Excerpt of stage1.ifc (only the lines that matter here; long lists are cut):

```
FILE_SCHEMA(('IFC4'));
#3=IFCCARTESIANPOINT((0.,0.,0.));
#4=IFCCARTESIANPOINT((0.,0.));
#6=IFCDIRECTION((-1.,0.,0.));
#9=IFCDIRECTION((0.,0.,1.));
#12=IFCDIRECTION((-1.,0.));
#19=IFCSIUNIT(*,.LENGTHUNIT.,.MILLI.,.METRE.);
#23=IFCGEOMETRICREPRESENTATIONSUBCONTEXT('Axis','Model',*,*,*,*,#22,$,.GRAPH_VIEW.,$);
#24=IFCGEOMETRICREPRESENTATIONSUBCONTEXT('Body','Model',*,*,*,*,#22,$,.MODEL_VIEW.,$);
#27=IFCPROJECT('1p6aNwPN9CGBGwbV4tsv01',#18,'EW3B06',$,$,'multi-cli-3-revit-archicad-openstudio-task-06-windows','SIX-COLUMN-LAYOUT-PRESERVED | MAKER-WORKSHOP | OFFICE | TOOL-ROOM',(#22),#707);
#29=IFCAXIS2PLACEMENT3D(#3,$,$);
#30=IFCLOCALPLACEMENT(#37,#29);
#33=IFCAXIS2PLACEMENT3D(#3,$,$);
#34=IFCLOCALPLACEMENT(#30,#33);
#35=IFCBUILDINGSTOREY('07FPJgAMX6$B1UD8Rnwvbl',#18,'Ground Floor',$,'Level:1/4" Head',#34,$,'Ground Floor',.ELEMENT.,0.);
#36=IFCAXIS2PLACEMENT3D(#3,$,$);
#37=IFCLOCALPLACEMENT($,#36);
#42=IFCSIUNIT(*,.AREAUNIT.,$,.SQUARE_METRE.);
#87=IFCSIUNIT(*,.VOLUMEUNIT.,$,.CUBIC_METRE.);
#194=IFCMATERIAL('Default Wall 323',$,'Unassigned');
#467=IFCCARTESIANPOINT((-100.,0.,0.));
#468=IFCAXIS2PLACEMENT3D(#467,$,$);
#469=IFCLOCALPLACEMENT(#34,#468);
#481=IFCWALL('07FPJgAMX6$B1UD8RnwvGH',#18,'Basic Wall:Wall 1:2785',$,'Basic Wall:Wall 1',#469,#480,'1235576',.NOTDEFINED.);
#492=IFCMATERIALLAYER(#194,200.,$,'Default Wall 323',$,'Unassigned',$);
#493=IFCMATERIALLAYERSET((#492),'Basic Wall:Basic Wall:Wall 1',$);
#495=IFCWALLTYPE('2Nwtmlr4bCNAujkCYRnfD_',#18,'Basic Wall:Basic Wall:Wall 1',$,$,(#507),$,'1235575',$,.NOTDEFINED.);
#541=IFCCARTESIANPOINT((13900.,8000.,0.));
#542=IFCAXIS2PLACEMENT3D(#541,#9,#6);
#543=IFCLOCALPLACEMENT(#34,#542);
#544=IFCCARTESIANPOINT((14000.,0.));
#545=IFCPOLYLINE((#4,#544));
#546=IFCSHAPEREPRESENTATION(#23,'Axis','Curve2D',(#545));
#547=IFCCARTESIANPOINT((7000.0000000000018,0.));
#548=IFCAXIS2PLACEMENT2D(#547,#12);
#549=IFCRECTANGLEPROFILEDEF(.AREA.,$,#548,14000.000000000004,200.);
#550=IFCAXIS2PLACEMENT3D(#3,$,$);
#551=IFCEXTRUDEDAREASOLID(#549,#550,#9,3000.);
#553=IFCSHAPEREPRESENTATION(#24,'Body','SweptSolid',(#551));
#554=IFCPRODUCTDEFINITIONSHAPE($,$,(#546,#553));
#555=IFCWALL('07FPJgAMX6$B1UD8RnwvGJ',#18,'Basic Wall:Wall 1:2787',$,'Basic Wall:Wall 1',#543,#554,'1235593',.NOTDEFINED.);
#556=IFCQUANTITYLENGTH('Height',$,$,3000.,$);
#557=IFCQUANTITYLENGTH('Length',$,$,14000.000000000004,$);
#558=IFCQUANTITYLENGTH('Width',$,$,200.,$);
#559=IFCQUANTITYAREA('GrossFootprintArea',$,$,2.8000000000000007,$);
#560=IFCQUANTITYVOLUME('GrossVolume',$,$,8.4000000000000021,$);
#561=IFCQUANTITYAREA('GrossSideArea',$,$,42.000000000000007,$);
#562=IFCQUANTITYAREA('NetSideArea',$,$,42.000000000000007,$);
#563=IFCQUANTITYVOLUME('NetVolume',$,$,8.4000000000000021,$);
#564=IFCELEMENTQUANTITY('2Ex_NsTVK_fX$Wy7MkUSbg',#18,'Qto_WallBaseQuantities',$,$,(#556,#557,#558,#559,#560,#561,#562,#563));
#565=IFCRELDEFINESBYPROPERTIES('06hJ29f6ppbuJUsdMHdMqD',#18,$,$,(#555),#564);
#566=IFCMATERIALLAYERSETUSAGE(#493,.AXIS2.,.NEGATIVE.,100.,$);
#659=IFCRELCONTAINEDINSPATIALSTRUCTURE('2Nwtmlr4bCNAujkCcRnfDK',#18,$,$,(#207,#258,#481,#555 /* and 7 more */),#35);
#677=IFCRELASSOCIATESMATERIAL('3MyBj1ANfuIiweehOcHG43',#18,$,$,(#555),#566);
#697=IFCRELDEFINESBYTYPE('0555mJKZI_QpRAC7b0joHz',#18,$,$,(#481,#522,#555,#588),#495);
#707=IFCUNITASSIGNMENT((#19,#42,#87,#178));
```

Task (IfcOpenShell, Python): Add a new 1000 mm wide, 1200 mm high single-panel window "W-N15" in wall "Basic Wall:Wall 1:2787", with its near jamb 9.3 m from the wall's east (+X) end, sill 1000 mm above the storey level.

```python
import numpy as np
import ifcopenshell
import ifcopenshell.api.feature
import ifcopenshell.api.geometry
import ifcopenshell.api.pset
import ifcopenshell.api.root
import ifcopenshell.api.spatial
import ifcopenshell.geom
import ifcopenshell.util.element
import ifcopenshell.util.placement
import ifcopenshell.util.representation
import ifcopenshell.util.shape
import ifcopenshell.util.unit

model = ifcopenshell.open("stage1.ifc")
unit_scale = ifcopenshell.util.unit.calculate_unit_scale(model)
area_scale = ifcopenshell.util.unit.calculate_unit_scale(model, "AREAUNIT")
volume_scale = ifcopenshell.util.unit.calculate_unit_scale(model, "VOLUMEUNIT")
settings = ifcopenshell.geom.settings()


def volume(element):
    """Net volume in cubic metres, openings subtracted."""
    shape = ifcopenshell.geom.create_shape(settings, element)
    return ifcopenshell.util.shape.get_volume(shape.geometry)


wall = model.by_id(555)
storey = ifcopenshell.util.element.get_container(wall, ifc_class="IfcBuildingStorey")
context = ifcopenshell.util.representation.get_context(model, "Model", "Body", "MODEL_VIEW")
before = volume(wall)

width, height, from_end, sill = 1, 1.2, 9.3, 1  # metres

# The wall runs along its own X axis, and the end named is its -X end.
wall_shape = ifcopenshell.geom.create_shape(settings, wall)
x, y, z = ifcopenshell.util.shape.get_vertices(wall_shape.geometry).T
start = x.min() + from_end
face, thickness = float(y.min()), float(y.max() - y.min())
wall_matrix = ifcopenshell.util.placement.get_local_placement(wall.ObjectPlacement)
level = ifcopenshell.util.placement.get_local_placement(storey.ObjectPlacement)[2, 3]


def in_wall(x, y):
    """Placement at x, y metres in the wall's axes, at sill height."""
    matrix = wall_matrix.copy()
    matrix[:, 3] = wall_matrix @ np.array([x / unit_scale, y / unit_scale, 0.0, 1.0])
    matrix[2, 3] = level + sill / unit_scale
    return matrix


# Opening: a box that overshoots both wall faces by 50 mm.
opening = ifcopenshell.api.root.create_entity(model, ifc_class="IfcOpeningElement", predefined_type="OPENING")
box = ifcopenshell.api.geometry.add_wall_representation(
    model, context=context, length=width, height=height, thickness=thickness + 0.1
)
ifcopenshell.api.geometry.assign_representation(model, product=opening, representation=box)
ifcopenshell.api.geometry.edit_object_placement(model, product=opening, matrix=in_wall(start, face - 0.05), is_si=False)
ifcopenshell.api.feature.add_feature(model, feature=opening, element=wall)

window = ifcopenshell.api.root.create_entity(model, ifc_class="IfcWindow", name="W-N15", predefined_type="WINDOW")
window.OverallWidth, window.OverallHeight = width / unit_scale, height / unit_scale
window.PartitioningType = "SINGLE_PANEL"
body = ifcopenshell.api.geometry.add_window_representation(
    model,
    context=context,
    overall_width=window.OverallWidth,
    overall_height=window.OverallHeight,
    partition_type="SINGLE_PANEL",
)
ifcopenshell.api.geometry.assign_representation(model, product=window, representation=body)
ifcopenshell.api.spatial.assign_container(model, products=[window], relating_structure=storey)
ifcopenshell.api.feature.add_filling(model, opening=opening, element=window)

# Centre the window in the wall's thickness.
ifcopenshell.api.geometry.edit_object_placement(model, product=window, matrix=in_wall(start, face), is_si=False)
window_shape = ifcopenshell.geom.create_shape(settings, window)
depth = ifcopenshell.util.shape.get_vertices(window_shape.geometry)[:, 1]
offset = face + thickness / 2 - (depth.min() + depth.max()) / 2
ifcopenshell.api.geometry.edit_object_placement(model, product=window, matrix=in_wall(start, offset), is_si=False)

after = volume(wall)

# Update the wall's stored quantities.
qto = model.by_id(ifcopenshell.util.element.get_pset(wall, "Qto_WallBaseQuantities", should_inherit=False)["id"])
ifcopenshell.api.pset.edit_qto(model, qto=qto, properties={
    "NetSideArea": after / thickness / area_scale,
    "NetVolume": after / volume_scale,
})

print(f"wall volume {before:.3f} -> {after:.3f} m3")

model.write("stage1-out.ifc")
```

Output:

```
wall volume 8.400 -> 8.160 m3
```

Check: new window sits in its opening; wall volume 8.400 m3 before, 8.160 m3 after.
